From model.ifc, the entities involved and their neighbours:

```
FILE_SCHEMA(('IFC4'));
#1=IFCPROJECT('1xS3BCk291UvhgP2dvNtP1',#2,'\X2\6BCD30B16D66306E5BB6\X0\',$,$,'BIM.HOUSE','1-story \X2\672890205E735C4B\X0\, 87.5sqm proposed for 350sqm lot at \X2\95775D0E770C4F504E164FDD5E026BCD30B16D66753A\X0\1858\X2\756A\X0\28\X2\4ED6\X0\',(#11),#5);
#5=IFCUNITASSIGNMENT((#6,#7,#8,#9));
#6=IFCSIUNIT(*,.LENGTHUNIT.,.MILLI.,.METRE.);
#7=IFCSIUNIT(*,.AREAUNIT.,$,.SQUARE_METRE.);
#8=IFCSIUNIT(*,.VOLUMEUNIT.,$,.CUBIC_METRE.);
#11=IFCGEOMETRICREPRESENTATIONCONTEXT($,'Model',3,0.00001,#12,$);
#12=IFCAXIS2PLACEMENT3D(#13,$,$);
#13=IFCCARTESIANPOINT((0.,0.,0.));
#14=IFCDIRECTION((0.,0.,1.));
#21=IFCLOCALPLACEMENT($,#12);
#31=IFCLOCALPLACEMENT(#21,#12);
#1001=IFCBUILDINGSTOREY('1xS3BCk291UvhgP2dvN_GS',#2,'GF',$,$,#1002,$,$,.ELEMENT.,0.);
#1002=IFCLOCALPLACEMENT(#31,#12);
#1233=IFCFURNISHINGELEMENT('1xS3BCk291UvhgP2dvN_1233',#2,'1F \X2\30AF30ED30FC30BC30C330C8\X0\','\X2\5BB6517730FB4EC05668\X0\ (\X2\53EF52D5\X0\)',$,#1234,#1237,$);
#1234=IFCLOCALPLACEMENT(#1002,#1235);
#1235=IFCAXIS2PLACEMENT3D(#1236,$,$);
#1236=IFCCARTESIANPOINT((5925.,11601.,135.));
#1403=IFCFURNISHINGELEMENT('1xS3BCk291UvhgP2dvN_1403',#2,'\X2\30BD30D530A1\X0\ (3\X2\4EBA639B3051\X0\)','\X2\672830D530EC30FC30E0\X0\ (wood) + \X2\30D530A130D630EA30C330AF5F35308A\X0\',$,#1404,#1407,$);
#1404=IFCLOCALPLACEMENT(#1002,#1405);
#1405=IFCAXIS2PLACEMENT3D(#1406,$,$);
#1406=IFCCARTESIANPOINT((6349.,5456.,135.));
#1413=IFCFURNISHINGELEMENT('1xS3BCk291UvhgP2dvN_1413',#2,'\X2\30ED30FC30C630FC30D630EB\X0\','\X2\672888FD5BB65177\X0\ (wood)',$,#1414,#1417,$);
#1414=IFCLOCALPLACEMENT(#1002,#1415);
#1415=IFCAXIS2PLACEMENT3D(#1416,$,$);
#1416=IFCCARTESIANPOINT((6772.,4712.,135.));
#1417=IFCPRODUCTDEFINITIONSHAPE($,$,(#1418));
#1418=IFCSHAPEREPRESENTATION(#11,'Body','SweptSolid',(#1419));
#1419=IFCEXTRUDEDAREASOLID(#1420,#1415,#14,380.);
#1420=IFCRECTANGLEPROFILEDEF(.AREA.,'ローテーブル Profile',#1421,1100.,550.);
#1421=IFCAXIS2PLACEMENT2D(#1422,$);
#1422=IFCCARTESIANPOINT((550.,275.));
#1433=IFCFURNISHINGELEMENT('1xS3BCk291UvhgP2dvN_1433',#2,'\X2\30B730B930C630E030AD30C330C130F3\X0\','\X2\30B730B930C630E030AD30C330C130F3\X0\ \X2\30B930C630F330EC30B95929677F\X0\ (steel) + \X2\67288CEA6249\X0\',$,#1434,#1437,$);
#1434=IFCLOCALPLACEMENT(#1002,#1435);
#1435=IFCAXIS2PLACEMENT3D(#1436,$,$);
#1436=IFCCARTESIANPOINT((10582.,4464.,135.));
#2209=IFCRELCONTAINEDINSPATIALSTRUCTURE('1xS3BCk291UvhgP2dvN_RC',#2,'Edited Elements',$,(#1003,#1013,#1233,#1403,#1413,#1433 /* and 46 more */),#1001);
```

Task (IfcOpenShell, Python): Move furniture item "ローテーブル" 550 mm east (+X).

```python
import ifcopenshell
import ifcopenshell.api.geometry
import ifcopenshell.util.placement

model = ifcopenshell.open("model.ifc")

item = model.by_guid("1xS3BCk291UvhgP2dvN_1413")
matrix = ifcopenshell.util.placement.get_local_placement(item.ObjectPlacement)
matrix[0, 3] += 550.0
ifcopenshell.api.geometry.edit_object_placement(model, product=item, matrix=matrix, is_si=False)

print(ifcopenshell.util.placement.get_local_placement(item.ObjectPlacement).round(3) + 0.0)

model.write("model-out.ifc")
```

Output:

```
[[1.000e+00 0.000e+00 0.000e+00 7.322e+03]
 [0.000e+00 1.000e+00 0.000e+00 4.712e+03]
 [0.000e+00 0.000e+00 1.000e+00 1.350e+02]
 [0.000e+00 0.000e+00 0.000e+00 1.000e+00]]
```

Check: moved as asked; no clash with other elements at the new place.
